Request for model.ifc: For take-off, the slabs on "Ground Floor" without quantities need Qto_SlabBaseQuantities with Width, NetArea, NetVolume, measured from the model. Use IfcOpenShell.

First a look at what the model holds.

```python
import ifcopenshell
import ifcopenshell.util.element
import ifcopenshell.util.unit

model = ifcopenshell.open("model.ifc")
print(model.schema)
for unit_type in ("LENGTHUNIT", "AREAUNIT", "VOLUMEUNIT"):
    print(unit_type, ifcopenshell.util.unit.calculate_unit_scale(model, unit_type))
storey = next(s for s in model.by_type("IfcBuildingStorey") if s.Name == "Ground Floor")
slabs = [e for e in ifcopenshell.util.element.get_decomposition(storey) if e.is_a("IfcSlab")]
for e in sorted(slabs, key=lambda e: e.id()):
    print(e.id(), e.is_a(), e.Name, list(ifcopenshell.util.element.get_psets(e, qtos_only=True)), sep=" | ")
```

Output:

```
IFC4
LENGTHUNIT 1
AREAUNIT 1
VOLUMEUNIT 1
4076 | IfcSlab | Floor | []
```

```python
import ifcopenshell
import ifcopenshell.api.pset
import ifcopenshell.geom
import ifcopenshell.util.element
import ifcopenshell.util.shape
import ifcopenshell.util.unit

model = ifcopenshell.open("model.ifc")
unit_scale = ifcopenshell.util.unit.calculate_unit_scale(model)
area_scale = ifcopenshell.util.unit.calculate_unit_scale(model, "AREAUNIT")
volume_scale = ifcopenshell.util.unit.calculate_unit_scale(model, "VOLUMEUNIT")
settings = ifcopenshell.geom.settings()

storey = next(s for s in model.by_type("IfcBuildingStorey") if s.Name == "Ground Floor")
slabs = [e for e in ifcopenshell.util.element.get_decomposition(storey) if e.is_a("IfcSlab")]

for e in sorted(slabs, key=lambda e: e.id()):
    if ifcopenshell.util.element.get_psets(e, qtos_only=True, should_inherit=False):
        continue
    # Geometry comes back in metres, in the element's own axes.
    shape = ifcopenshell.geom.create_shape(settings, e)
    values = {
        "Width": ifcopenshell.util.shape.get_z(shape.geometry) / unit_scale,
        "NetArea": ifcopenshell.util.shape.get_footprint_area(shape.geometry) / area_scale,
        "NetVolume": ifcopenshell.util.shape.get_volume(shape.geometry) / volume_scale,
    }
    qto = ifcopenshell.api.pset.add_qto(model, product=e, name="Qto_SlabBaseQuantities")
    ifcopenshell.api.pset.edit_qto(model, qto=qto, properties=values)
    print(e.id(), {k: round(v, 3) for k, v in values.items()})

model.write("model_updated.ifc")
```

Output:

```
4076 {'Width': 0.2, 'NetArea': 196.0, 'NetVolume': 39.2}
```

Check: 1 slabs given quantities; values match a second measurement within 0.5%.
